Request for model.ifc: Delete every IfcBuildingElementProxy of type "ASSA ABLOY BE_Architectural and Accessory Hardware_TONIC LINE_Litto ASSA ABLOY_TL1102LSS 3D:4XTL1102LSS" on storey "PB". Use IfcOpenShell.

First a look at what the model holds.

```python
import ifcopenshell
import ifcopenshell.util.element

model = ifcopenshell.open("model.ifc")
print(model.schema)
storey = next(s for s in model.by_type("IfcBuildingStorey") if s.Name == "PB")
proxies = [e for e in ifcopenshell.util.element.get_decomposition(storey) if e.is_a("IfcBuildingElementProxy")]
seen = {}
for e in proxies:
    element_type = ifcopenshell.util.element.get_type(e)
    name = element_type.Name if element_type not in (None, e) else None
    seen[name] = seen.get(name, 0) + 1
for name, count in sorted(seen.items(), key=str):
    print(count, "x", name)
```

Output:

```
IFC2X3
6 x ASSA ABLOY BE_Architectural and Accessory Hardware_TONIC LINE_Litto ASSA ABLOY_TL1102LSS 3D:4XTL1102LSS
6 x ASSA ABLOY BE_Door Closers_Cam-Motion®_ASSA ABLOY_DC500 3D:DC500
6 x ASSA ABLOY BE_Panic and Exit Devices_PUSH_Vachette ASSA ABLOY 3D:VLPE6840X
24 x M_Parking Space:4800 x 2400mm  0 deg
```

```python
import ifcopenshell
import ifcopenshell.api.root
import ifcopenshell.util.element

model = ifcopenshell.open("model.ifc")

storey = next(s for s in model.by_type("IfcBuildingStorey") if s.Name == "PB")
proxies = [e for e in ifcopenshell.util.element.get_decomposition(storey) if e.is_a("IfcBuildingElementProxy")]
targets = [e for e in proxies if (t := ifcopenshell.util.element.get_type(e)) not in (None, e) and t.Name == "ASSA ABLOY BE_Architectural and Accessory Hardware_TONIC LINE_Litto ASSA ABLOY_TL1102LSS 3D:4XTL1102LSS"]

for e in targets:
    ifcopenshell.api.root.remove_product(model, product=e)
print(len(targets), "removed")

model.write("model_edited.ifc")
```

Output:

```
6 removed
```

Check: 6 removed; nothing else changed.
